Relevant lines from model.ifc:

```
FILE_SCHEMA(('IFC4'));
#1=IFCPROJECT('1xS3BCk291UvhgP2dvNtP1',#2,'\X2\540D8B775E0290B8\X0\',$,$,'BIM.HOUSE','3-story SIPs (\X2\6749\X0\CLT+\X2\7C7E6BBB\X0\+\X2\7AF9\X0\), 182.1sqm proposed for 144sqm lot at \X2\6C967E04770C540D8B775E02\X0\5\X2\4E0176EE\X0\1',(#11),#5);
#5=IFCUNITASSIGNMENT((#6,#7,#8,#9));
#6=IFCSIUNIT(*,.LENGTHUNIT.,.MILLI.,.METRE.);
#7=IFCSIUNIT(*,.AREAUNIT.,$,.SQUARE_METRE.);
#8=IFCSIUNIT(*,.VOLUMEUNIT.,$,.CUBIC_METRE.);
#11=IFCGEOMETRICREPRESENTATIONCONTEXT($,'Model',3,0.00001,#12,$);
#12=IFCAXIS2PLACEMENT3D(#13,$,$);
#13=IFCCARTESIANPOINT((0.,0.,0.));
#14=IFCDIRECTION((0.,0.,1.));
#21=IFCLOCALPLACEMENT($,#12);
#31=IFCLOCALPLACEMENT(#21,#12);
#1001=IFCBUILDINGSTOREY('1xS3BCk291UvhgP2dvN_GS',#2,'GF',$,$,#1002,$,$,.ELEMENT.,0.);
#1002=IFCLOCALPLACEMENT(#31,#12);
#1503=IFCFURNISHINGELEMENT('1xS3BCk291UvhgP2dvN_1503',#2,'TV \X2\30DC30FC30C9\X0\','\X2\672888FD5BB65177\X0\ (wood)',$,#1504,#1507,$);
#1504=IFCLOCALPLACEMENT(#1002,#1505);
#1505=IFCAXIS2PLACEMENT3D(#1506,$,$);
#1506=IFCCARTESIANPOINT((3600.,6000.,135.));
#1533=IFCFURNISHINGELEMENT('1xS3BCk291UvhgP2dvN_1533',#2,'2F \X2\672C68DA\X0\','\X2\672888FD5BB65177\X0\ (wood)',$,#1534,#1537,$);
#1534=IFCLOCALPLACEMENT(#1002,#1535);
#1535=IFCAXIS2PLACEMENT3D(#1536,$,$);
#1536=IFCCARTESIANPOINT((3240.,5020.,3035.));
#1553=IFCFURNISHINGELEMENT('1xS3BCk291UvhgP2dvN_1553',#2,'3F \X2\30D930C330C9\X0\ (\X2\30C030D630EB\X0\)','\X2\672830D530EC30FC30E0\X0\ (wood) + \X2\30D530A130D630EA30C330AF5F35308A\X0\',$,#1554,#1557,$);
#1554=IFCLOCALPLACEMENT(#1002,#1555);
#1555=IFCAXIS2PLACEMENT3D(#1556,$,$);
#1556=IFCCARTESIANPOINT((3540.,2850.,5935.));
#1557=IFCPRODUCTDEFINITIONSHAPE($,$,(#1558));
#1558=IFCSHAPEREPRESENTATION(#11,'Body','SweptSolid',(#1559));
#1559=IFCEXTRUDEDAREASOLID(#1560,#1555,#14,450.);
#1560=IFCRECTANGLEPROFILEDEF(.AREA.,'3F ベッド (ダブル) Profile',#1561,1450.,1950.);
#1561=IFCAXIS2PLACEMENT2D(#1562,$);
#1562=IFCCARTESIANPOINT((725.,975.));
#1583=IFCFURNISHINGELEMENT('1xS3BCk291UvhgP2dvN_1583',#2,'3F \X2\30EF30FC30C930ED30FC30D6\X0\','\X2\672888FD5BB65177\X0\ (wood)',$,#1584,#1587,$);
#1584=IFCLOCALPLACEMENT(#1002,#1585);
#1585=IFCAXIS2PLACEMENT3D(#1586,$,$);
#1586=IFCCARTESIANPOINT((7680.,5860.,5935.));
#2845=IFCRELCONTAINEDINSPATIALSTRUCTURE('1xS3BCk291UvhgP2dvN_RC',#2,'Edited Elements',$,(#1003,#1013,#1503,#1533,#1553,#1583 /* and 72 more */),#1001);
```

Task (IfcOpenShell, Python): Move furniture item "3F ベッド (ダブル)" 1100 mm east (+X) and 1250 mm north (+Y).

```python
import ifcopenshell
import ifcopenshell.api.geometry
import ifcopenshell.util.placement
import ifcopenshell.util.unit

model = ifcopenshell.open("model.ifc")
unit_scale = ifcopenshell.util.unit.calculate_unit_scale(model)

item = model.by_guid("1xS3BCk291UvhgP2dvN_1553")
matrix = ifcopenshell.util.placement.get_local_placement(item.ObjectPlacement)
matrix[0, 3] += 1.1 / unit_scale
matrix[1, 3] += 1.25 / unit_scale
ifcopenshell.api.geometry.edit_object_placement(model, product=item, matrix=matrix, is_si=False)

print(ifcopenshell.util.placement.get_local_placement(item.ObjectPlacement).round(3) + 0.0)

model.write("model_rev.ifc")
```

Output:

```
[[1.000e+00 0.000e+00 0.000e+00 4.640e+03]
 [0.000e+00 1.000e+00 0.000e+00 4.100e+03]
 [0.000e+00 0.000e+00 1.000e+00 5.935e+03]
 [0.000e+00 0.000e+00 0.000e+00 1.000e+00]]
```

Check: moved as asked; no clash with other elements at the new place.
